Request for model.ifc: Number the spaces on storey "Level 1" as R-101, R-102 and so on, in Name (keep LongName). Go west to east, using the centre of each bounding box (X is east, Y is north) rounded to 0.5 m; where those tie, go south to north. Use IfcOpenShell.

First a look at what the model holds.

```python
import ifcopenshell
import ifcopenshell.util.element
import ifcopenshell.util.placement

model = ifcopenshell.open("model.ifc")
print(model.schema)
storey = next(s for s in model.by_type("IfcBuildingStorey") if s.Name == "Level 1")
spaces = [e for e in ifcopenshell.util.element.get_decomposition(storey) if e.is_a("IfcSpace")]
for e in sorted(spaces, key=lambda e: e.id()):
    origin = ifcopenshell.util.placement.get_local_placement(e.ObjectPlacement)[:3, 3]
    print(e.id(), e.Name, e.LongName, origin.round(2) + 0.0, sep=" | ")
```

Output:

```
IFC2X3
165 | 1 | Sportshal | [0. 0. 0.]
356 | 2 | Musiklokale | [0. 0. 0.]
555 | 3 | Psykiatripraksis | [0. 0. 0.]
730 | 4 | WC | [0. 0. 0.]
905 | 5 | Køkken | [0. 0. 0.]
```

```python
import ifcopenshell
import ifcopenshell.geom
import ifcopenshell.util.element
import ifcopenshell.util.shape

model = ifcopenshell.open("model.ifc")
settings = ifcopenshell.geom.settings()
settings.set("use-world-coords", True)


def centre(element):
    shape = ifcopenshell.geom.create_shape(settings, element)
    return ifcopenshell.util.shape.get_bbox_centroid(shape.geometry)


storey = next(s for s in model.by_type("IfcBuildingStorey") if s.Name == "Level 1")
spaces = [e for e in ifcopenshell.util.element.get_decomposition(storey) if e.is_a("IfcSpace")]

# Insertion points can sit at a corner or the storey origin, so sort by the geometry (in metres).
centres = {e: centre(e) for e in spaces}
spaces.sort(key=lambda e: (round(centres[e][0] / 0.5), centres[e][1]))

for i, e in enumerate(spaces, start=1):
    number = f"R-1{i:02d}"
    e.Name = number
    print(e.id(), number)

model.write("model_edited.ifc")
```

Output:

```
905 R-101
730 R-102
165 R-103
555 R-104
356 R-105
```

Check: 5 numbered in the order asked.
